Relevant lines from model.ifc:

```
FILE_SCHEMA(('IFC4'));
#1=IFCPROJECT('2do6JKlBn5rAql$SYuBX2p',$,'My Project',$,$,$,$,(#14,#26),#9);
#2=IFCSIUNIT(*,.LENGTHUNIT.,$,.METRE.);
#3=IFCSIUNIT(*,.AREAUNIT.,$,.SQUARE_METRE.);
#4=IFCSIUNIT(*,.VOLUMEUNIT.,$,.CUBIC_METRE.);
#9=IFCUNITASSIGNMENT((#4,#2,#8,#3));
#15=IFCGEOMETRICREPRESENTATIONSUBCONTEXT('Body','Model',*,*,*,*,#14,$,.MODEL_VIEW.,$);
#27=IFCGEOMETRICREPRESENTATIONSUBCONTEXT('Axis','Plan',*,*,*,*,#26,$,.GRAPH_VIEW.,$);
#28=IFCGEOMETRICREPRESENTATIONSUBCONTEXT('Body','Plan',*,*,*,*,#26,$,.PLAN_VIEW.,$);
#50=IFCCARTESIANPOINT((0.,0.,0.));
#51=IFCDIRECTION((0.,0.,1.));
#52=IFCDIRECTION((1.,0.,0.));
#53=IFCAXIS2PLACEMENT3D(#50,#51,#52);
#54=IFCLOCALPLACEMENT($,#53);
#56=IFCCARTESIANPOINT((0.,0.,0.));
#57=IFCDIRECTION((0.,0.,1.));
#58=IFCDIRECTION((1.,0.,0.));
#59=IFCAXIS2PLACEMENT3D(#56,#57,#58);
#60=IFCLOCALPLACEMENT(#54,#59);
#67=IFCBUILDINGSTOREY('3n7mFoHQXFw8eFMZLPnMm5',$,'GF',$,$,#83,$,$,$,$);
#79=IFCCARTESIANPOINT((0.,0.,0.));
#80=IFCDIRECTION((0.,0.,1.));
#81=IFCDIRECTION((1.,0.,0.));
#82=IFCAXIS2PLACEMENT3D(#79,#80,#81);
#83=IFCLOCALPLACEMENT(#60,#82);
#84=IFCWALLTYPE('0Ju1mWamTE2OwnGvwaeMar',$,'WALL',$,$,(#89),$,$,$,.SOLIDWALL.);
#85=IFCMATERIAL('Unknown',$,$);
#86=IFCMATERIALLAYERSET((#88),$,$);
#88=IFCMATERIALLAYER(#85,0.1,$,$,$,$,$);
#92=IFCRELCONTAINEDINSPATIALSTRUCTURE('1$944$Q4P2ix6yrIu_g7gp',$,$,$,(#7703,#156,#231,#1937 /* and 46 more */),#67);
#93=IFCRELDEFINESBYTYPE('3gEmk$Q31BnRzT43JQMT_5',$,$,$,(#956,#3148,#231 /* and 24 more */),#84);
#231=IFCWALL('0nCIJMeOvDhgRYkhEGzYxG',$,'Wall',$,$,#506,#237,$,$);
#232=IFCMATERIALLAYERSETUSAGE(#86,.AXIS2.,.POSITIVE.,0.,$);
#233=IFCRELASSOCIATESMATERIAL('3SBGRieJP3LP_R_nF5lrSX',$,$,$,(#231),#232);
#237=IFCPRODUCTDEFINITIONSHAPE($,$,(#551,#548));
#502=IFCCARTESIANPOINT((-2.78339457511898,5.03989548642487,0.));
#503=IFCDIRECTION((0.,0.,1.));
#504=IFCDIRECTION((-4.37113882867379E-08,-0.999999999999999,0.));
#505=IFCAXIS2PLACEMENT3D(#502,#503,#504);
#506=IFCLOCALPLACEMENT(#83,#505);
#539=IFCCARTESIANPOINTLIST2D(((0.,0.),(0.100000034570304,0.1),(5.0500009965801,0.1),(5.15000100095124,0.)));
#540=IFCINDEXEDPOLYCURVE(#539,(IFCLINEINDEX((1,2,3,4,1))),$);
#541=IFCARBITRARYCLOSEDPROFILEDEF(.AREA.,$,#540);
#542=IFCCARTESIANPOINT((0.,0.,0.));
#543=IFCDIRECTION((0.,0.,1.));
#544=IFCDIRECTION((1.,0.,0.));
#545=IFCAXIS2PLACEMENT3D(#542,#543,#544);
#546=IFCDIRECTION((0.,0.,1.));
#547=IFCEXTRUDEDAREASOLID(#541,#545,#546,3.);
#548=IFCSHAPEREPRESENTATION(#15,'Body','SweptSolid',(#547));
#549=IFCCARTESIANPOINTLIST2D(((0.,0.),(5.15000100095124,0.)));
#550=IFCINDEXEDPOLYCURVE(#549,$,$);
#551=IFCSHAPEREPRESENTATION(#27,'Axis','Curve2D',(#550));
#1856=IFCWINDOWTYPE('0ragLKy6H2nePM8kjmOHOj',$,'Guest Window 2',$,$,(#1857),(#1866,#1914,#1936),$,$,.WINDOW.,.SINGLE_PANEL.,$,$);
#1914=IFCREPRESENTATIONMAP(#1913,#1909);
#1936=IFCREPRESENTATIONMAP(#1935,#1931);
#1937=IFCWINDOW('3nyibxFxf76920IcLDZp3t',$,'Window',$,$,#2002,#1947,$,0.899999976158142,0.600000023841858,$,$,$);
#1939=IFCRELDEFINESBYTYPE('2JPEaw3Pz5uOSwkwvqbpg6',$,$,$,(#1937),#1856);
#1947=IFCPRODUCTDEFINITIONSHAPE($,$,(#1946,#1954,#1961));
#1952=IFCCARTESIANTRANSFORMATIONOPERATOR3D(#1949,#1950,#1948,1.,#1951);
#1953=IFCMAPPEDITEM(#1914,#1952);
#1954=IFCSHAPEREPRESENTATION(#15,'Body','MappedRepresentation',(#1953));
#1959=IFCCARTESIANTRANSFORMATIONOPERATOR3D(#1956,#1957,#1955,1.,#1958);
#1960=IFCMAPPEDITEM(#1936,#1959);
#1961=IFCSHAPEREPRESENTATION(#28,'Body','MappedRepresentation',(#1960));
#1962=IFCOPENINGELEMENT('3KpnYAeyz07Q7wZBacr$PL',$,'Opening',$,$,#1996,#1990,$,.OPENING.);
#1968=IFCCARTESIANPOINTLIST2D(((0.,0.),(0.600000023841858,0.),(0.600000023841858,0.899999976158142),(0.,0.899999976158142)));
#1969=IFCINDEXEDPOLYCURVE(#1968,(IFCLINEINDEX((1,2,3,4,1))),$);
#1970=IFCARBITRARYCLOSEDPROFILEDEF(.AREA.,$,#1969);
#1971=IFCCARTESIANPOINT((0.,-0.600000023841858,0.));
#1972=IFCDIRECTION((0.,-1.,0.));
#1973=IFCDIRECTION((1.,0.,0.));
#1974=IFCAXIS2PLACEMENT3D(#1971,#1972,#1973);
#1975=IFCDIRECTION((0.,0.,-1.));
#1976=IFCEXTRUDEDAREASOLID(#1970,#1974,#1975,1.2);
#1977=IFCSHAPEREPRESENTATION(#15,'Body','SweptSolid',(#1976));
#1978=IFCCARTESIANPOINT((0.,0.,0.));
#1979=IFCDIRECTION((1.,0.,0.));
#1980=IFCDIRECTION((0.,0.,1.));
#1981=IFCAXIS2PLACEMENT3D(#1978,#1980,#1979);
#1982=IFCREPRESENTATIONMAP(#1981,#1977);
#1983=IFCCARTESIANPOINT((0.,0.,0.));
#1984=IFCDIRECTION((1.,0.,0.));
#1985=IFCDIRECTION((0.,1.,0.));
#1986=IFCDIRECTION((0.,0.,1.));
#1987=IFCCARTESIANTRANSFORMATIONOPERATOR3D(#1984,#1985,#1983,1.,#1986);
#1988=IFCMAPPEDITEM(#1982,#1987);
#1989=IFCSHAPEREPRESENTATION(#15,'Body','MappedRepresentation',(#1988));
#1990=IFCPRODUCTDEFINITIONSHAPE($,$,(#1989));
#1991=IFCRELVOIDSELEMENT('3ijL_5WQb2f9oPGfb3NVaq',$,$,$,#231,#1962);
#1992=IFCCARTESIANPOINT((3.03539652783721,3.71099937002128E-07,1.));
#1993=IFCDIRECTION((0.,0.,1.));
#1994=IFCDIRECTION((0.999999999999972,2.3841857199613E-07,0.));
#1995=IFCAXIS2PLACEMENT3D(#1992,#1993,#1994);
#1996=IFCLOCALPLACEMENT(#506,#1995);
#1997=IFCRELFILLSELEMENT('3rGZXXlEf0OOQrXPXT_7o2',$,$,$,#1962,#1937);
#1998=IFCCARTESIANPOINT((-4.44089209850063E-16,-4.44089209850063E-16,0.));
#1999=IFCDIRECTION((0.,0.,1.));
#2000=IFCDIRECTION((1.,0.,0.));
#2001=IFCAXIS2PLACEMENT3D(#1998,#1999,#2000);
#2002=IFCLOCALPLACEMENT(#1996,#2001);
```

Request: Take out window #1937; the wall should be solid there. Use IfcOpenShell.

```python
import ifcopenshell
import ifcopenshell.api.feature
import ifcopenshell.api.root
import ifcopenshell.geom
import ifcopenshell.util.shape

model = ifcopenshell.open("model.ifc")
settings = ifcopenshell.geom.settings()


def volume(element):
    """Net volume in cubic metres, openings subtracted."""
    shape = ifcopenshell.geom.create_shape(settings, element)
    return ifcopenshell.util.shape.get_volume(shape.geometry)


window = model.by_guid("3nyibxFxf76920IcLDZp3t")
opening = window.FillsVoids[0].RelatingOpeningElement
wall = opening.VoidsElements[0].RelatingBuildingElement
before = volume(wall)

ifcopenshell.api.root.remove_product(model, product=window)
ifcopenshell.api.feature.remove_feature(model, feature=opening)

after = volume(wall)

print(f"wall volume {before:.3f} -> {after:.3f} m3")

model.write("model_edited.ifc")
```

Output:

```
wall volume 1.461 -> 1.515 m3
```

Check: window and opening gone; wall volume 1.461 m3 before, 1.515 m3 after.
